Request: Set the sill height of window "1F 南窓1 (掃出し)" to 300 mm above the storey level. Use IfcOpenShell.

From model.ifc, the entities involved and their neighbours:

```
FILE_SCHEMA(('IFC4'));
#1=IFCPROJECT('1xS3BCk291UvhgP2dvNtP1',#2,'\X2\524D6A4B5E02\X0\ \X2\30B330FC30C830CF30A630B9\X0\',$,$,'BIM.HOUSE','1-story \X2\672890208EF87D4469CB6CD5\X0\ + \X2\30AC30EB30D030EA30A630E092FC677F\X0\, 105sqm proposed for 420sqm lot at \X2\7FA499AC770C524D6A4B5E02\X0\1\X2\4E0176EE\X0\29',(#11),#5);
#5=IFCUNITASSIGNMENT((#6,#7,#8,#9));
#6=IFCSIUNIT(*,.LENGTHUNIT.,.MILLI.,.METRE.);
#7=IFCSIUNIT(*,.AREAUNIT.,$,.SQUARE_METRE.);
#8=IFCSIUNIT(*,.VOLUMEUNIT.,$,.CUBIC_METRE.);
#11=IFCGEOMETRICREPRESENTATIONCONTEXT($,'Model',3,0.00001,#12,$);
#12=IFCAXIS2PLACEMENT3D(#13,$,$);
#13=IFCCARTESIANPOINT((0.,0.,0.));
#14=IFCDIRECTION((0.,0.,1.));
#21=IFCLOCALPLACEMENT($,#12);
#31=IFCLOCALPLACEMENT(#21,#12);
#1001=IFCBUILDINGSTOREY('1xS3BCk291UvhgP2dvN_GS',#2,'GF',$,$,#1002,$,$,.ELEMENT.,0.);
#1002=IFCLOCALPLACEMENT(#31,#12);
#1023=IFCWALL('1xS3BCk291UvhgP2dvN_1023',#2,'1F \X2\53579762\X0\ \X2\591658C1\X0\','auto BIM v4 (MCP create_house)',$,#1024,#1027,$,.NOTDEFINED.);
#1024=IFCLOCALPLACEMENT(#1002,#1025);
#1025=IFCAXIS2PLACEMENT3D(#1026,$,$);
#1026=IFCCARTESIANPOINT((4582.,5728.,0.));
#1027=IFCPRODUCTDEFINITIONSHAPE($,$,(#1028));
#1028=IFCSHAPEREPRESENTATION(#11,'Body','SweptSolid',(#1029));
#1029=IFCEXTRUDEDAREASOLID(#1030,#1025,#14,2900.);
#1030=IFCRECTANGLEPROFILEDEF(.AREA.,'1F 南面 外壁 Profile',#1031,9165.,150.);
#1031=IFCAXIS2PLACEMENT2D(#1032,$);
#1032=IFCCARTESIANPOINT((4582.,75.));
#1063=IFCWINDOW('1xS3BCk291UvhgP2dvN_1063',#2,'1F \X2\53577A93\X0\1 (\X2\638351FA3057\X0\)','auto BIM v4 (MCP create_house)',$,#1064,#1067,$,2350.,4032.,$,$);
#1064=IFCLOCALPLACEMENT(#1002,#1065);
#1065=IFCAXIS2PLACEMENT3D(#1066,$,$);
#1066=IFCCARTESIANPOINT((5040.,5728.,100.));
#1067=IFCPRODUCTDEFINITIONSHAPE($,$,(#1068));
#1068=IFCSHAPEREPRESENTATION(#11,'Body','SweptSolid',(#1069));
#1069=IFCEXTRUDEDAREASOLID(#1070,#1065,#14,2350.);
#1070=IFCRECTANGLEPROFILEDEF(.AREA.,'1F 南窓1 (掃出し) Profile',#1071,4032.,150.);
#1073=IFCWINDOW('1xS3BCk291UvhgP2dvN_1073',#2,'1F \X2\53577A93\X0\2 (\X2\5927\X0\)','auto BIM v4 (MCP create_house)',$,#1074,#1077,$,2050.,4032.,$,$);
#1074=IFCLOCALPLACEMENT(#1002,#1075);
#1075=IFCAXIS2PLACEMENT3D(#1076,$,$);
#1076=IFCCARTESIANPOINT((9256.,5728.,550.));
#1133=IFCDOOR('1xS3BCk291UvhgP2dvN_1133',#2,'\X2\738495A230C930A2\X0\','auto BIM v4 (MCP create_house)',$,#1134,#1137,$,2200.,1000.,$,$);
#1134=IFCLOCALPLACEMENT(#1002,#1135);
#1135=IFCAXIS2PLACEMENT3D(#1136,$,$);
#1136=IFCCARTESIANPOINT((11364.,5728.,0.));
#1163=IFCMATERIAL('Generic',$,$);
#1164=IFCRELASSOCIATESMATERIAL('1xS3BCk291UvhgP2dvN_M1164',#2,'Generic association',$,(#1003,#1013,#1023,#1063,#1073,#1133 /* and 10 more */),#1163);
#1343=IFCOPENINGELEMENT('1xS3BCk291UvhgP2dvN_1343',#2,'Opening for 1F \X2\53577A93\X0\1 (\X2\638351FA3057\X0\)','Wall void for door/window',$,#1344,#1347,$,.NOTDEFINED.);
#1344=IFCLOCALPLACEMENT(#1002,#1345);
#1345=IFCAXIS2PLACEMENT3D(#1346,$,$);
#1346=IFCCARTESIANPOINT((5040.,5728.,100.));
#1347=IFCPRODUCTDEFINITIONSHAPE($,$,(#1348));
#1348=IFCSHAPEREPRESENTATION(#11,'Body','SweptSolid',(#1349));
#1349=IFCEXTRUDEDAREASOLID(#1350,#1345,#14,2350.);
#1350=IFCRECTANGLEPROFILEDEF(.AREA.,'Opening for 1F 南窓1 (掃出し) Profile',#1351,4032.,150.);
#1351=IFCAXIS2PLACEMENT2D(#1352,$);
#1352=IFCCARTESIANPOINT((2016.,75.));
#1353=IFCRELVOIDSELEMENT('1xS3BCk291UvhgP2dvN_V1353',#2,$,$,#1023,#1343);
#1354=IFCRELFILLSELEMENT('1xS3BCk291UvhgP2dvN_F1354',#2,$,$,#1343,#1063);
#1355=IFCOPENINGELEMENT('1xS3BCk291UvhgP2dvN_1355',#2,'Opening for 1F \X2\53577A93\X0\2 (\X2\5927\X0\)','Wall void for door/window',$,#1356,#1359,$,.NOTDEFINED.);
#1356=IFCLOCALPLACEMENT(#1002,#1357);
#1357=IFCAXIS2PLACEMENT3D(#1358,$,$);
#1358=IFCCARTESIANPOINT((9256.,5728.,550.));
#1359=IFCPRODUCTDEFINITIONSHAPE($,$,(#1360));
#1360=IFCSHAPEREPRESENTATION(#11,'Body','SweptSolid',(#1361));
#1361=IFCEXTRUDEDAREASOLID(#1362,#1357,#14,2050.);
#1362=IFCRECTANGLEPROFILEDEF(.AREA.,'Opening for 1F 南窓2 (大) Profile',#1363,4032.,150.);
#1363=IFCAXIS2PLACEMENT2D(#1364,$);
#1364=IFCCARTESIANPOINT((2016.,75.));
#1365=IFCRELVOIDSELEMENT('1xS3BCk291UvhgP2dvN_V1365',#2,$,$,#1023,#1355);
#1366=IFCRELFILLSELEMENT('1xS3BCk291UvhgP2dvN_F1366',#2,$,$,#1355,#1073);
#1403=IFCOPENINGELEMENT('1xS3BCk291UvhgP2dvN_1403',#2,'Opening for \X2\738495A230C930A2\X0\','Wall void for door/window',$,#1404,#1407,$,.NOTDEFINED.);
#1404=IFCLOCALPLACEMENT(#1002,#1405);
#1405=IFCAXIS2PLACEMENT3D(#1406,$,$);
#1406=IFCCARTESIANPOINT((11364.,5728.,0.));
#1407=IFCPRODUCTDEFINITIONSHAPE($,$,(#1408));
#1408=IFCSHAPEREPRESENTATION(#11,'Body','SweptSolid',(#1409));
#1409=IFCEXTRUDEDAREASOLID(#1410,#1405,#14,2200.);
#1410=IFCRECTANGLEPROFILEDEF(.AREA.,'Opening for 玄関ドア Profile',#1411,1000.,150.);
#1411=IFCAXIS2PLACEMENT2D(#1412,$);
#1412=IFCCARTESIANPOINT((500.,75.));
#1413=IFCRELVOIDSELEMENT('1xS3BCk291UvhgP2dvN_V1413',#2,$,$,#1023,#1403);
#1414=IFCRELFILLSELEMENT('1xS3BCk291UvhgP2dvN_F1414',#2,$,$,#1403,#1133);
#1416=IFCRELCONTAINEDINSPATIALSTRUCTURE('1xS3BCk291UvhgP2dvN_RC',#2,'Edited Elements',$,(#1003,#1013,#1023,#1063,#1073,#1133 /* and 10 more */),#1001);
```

```python
import numpy as np
import ifcopenshell
import ifcopenshell.api.geometry
import ifcopenshell.geom
import ifcopenshell.util.element
import ifcopenshell.util.placement
import ifcopenshell.util.shape
import ifcopenshell.util.unit

model = ifcopenshell.open("model.ifc")
unit_scale = ifcopenshell.util.unit.calculate_unit_scale(model)

window = model.by_id(1063)
opening = window.FillsVoids[0].RelatingOpeningElement
storey = ifcopenshell.util.element.get_container(window, ifc_class="IfcBuildingStorey")
level = ifcopenshell.util.placement.get_local_placement(storey.ObjectPlacement)[2, 3]

# The opening's origin need not be at the sill, so measure its lowest point.
shape = ifcopenshell.geom.create_shape(ifcopenshell.geom.settings(), opening)
bottom = ifcopenshell.util.shape.get_shape_bottom_elevation(shape, shape.geometry) / unit_scale
dz = level + 0.3 / unit_scale - bottom

shift = np.array([0.0, 0.0, dz])
# The window is not placed relative to its opening, so move both.
for product in (opening, window):
    matrix = ifcopenshell.util.placement.get_local_placement(product.ObjectPlacement)
    matrix[:3, 3] += shift
    ifcopenshell.api.geometry.edit_object_placement(model, product=product, matrix=matrix, is_si=False)

print(f"moved by {dz * unit_scale:+.3f} m")

model.write("model-out.ifc")
```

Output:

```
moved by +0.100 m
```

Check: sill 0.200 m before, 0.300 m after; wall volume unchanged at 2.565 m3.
